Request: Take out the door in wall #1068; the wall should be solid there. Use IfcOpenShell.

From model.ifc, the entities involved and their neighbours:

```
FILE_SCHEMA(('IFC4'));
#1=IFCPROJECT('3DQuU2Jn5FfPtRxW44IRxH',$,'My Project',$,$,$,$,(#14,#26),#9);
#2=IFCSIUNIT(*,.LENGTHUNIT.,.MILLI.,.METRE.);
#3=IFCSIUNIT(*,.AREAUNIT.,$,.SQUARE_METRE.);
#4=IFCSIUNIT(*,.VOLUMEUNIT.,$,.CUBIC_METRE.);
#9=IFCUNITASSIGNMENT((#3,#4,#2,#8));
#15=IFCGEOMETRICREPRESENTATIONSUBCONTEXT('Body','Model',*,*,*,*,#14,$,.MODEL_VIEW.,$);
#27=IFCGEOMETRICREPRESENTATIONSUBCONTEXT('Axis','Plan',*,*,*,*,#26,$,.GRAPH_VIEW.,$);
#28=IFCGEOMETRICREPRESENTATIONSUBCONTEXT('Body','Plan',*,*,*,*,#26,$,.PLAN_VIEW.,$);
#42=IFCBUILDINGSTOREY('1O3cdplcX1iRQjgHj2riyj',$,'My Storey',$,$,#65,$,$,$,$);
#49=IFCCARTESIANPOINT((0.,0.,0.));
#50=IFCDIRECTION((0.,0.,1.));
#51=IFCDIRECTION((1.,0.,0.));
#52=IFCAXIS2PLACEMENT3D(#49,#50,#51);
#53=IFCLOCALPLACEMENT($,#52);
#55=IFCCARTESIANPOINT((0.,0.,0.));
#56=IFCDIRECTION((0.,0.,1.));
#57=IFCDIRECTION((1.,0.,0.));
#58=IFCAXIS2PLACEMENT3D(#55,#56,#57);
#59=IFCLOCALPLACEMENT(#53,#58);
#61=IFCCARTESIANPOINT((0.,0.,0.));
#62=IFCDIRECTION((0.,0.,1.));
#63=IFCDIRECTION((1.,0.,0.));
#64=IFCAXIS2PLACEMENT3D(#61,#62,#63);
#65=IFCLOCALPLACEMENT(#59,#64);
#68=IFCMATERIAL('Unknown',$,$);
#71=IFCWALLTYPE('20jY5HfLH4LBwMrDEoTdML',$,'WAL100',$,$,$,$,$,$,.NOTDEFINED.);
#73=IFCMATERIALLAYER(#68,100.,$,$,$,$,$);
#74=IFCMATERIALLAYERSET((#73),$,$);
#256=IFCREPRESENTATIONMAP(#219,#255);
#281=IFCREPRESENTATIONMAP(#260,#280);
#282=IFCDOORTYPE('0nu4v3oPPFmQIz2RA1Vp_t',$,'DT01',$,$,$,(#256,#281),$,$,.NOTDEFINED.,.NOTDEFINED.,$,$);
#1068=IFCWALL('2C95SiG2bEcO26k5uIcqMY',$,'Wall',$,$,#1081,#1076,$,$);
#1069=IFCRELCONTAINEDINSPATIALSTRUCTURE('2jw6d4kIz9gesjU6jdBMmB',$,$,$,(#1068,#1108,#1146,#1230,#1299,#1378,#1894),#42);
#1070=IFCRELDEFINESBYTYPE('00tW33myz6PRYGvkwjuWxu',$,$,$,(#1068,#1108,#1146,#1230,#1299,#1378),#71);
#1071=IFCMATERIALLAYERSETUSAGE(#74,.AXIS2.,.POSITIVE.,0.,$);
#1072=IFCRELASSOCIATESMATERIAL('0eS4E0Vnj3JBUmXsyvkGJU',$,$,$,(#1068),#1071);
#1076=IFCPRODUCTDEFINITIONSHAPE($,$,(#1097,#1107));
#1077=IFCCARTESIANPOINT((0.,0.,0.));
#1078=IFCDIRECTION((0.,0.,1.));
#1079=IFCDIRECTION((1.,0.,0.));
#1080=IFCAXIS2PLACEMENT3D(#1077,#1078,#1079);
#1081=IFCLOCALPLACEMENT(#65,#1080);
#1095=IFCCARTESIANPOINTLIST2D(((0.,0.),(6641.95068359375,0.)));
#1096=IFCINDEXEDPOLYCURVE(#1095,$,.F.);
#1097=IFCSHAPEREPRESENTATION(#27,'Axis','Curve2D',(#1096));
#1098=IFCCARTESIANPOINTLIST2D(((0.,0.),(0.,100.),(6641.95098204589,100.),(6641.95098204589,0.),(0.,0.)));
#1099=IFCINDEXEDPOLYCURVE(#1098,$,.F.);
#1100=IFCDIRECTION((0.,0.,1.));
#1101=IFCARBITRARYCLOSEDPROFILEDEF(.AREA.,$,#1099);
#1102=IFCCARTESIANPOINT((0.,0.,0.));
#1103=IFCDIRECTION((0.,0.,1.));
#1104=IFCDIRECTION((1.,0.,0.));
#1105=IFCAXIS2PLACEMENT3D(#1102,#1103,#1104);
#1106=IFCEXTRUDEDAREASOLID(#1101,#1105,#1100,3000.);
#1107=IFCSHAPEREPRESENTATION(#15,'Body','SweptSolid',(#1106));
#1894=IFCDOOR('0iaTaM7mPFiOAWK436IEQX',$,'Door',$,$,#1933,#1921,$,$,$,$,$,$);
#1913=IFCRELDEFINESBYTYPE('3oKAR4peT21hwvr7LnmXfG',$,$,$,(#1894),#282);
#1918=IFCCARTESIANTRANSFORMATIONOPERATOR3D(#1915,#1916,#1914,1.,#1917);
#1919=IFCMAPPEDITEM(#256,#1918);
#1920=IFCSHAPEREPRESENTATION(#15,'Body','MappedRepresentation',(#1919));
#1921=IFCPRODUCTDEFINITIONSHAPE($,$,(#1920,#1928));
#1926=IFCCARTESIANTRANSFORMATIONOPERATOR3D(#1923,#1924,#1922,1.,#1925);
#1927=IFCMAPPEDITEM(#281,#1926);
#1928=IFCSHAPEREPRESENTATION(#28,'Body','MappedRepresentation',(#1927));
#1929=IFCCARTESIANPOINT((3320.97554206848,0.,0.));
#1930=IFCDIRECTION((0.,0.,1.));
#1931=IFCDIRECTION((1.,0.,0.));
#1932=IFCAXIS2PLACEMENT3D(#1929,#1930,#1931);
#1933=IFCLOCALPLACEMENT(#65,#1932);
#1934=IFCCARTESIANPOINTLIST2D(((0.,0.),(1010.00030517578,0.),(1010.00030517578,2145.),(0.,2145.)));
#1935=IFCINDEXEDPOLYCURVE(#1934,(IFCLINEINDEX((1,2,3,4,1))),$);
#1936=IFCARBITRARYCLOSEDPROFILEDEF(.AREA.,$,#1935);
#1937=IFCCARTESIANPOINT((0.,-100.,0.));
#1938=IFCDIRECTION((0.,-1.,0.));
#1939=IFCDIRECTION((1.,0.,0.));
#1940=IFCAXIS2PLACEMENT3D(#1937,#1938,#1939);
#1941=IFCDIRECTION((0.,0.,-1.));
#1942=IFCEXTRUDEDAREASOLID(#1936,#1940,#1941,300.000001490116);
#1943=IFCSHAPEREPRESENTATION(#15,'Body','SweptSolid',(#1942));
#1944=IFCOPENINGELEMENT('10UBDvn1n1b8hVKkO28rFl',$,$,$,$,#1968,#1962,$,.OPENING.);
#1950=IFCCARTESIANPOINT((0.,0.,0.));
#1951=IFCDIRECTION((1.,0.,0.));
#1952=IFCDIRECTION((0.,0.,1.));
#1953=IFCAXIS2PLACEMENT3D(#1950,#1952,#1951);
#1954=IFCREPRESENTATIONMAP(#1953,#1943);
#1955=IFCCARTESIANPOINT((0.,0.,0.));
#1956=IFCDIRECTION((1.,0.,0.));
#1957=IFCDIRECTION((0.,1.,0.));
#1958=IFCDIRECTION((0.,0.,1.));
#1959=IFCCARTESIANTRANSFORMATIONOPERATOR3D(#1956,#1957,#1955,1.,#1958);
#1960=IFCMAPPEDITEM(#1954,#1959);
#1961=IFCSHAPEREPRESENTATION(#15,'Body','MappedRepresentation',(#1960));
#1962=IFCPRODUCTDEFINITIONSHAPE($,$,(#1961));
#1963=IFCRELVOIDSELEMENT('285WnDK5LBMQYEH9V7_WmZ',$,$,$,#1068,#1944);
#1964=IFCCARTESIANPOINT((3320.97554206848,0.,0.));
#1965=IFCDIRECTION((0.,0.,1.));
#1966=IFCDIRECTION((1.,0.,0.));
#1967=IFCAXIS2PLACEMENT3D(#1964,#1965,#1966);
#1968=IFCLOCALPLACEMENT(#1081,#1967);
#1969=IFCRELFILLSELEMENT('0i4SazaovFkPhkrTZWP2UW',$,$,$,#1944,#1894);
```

```python
import ifcopenshell
import ifcopenshell.api.feature
import ifcopenshell.api.root
import ifcopenshell.geom
import ifcopenshell.util.shape

model = ifcopenshell.open("model.ifc")
settings = ifcopenshell.geom.settings()


def volume(element):
    """Net volume in cubic metres, openings subtracted."""
    shape = ifcopenshell.geom.create_shape(settings, element)
    return ifcopenshell.util.shape.get_volume(shape.geometry)


door = model.by_guid("0iaTaM7mPFiOAWK436IEQX")
opening = door.FillsVoids[0].RelatingOpeningElement
wall = opening.VoidsElements[0].RelatingBuildingElement
before = volume(wall)

ifcopenshell.api.root.remove_product(model, product=door)
ifcopenshell.api.feature.remove_feature(model, feature=opening)

after = volume(wall)

print(f"wall volume {before:.3f} -> {after:.3f} m3")

model.write("model_edited.ifc")
```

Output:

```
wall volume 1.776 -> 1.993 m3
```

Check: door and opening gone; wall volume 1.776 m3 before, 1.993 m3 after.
